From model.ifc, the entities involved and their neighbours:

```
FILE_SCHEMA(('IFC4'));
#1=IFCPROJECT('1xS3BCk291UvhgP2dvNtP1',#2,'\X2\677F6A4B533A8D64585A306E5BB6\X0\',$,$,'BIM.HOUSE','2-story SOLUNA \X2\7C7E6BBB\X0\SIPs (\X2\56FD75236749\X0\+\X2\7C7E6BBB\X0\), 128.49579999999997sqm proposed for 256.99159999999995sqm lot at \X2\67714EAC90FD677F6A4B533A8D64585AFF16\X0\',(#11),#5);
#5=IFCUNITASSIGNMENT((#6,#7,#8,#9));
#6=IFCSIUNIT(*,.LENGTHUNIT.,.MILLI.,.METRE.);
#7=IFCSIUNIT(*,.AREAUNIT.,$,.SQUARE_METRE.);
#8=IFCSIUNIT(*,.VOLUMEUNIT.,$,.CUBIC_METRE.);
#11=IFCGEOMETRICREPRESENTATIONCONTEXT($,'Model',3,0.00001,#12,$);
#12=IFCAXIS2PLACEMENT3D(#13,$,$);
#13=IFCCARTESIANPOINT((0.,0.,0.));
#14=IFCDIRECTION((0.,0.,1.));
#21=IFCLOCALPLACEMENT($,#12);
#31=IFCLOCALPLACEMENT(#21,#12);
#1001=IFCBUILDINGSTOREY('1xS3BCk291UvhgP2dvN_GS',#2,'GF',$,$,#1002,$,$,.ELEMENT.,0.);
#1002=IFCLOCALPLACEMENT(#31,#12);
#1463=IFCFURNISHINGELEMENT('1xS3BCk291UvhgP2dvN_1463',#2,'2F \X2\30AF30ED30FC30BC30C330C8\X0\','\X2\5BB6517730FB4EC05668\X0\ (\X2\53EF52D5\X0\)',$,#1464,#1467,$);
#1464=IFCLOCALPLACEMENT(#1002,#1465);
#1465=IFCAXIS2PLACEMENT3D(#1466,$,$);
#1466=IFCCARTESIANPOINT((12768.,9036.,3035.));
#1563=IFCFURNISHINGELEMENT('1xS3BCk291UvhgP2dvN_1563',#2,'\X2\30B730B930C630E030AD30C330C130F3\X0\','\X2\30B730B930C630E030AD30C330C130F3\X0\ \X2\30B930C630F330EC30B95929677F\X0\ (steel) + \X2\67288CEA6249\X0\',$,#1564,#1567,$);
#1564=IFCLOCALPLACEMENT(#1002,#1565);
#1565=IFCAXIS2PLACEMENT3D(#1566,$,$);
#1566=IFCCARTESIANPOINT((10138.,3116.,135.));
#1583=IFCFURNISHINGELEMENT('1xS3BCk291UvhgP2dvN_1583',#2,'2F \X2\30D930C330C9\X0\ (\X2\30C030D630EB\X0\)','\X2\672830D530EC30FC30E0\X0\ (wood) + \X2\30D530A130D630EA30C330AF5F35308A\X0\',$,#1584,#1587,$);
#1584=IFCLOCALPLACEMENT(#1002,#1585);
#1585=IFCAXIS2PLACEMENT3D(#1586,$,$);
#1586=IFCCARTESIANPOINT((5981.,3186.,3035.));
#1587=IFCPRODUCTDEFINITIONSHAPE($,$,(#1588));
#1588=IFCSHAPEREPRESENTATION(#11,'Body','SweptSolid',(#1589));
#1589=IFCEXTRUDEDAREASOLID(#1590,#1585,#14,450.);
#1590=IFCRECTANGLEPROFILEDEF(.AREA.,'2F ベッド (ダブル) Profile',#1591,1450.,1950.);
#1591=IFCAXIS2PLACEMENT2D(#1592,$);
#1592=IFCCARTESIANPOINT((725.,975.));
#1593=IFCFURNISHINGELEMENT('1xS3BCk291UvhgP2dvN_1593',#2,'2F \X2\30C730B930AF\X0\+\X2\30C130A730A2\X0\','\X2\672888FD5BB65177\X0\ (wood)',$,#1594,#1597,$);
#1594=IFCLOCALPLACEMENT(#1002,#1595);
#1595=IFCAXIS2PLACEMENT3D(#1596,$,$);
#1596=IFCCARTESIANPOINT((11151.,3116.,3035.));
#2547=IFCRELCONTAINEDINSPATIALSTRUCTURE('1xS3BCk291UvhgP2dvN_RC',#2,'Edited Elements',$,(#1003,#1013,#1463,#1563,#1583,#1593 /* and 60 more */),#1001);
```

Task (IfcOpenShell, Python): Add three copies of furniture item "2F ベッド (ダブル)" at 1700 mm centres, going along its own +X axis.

```python
import ifcopenshell
import ifcopenshell.api.geometry
import ifcopenshell.api.root
import ifcopenshell.util.element
import ifcopenshell.util.placement

model = ifcopenshell.open("model.ifc")


def reuse_history(source, copy):
    """copy_class also copies each property set's owner history, people and application; keep the originals."""
    for rel in copy.IsDefinedBy:
        if rel.is_a("IfcRelDefinesByProperties") and (history := rel.RelatingPropertyDefinition.OwnerHistory):
            rel.RelatingPropertyDefinition.OwnerHistory = source.OwnerHistory
            ifcopenshell.util.element.remove_deep2(model, history)


source = model.by_guid("1xS3BCk291UvhgP2dvN_1583")
base = ifcopenshell.util.placement.get_local_placement(source.ObjectPlacement)
step = base[:3, 0] * 1700.0

for i in range(1, 4):
    copy = ifcopenshell.api.root.copy_class(model, product=source)
    copy.Representation = ifcopenshell.util.element.copy_deep(
        model, source.Representation, exclude=["IfcGeometricRepresentationContext", "IfcRepresentationMap"]
    )
    reuse_history(source, copy)
    matrix = base.copy()
    matrix[:3, 3] += i * step
    print("added at", matrix[:3, 3].round(3) + 0.0)
    ifcopenshell.api.geometry.edit_object_placement(model, product=copy, matrix=matrix, is_si=False)

model.write("model-out.ifc")
```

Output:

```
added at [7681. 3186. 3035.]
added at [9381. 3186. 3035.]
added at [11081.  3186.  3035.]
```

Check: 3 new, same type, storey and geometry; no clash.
